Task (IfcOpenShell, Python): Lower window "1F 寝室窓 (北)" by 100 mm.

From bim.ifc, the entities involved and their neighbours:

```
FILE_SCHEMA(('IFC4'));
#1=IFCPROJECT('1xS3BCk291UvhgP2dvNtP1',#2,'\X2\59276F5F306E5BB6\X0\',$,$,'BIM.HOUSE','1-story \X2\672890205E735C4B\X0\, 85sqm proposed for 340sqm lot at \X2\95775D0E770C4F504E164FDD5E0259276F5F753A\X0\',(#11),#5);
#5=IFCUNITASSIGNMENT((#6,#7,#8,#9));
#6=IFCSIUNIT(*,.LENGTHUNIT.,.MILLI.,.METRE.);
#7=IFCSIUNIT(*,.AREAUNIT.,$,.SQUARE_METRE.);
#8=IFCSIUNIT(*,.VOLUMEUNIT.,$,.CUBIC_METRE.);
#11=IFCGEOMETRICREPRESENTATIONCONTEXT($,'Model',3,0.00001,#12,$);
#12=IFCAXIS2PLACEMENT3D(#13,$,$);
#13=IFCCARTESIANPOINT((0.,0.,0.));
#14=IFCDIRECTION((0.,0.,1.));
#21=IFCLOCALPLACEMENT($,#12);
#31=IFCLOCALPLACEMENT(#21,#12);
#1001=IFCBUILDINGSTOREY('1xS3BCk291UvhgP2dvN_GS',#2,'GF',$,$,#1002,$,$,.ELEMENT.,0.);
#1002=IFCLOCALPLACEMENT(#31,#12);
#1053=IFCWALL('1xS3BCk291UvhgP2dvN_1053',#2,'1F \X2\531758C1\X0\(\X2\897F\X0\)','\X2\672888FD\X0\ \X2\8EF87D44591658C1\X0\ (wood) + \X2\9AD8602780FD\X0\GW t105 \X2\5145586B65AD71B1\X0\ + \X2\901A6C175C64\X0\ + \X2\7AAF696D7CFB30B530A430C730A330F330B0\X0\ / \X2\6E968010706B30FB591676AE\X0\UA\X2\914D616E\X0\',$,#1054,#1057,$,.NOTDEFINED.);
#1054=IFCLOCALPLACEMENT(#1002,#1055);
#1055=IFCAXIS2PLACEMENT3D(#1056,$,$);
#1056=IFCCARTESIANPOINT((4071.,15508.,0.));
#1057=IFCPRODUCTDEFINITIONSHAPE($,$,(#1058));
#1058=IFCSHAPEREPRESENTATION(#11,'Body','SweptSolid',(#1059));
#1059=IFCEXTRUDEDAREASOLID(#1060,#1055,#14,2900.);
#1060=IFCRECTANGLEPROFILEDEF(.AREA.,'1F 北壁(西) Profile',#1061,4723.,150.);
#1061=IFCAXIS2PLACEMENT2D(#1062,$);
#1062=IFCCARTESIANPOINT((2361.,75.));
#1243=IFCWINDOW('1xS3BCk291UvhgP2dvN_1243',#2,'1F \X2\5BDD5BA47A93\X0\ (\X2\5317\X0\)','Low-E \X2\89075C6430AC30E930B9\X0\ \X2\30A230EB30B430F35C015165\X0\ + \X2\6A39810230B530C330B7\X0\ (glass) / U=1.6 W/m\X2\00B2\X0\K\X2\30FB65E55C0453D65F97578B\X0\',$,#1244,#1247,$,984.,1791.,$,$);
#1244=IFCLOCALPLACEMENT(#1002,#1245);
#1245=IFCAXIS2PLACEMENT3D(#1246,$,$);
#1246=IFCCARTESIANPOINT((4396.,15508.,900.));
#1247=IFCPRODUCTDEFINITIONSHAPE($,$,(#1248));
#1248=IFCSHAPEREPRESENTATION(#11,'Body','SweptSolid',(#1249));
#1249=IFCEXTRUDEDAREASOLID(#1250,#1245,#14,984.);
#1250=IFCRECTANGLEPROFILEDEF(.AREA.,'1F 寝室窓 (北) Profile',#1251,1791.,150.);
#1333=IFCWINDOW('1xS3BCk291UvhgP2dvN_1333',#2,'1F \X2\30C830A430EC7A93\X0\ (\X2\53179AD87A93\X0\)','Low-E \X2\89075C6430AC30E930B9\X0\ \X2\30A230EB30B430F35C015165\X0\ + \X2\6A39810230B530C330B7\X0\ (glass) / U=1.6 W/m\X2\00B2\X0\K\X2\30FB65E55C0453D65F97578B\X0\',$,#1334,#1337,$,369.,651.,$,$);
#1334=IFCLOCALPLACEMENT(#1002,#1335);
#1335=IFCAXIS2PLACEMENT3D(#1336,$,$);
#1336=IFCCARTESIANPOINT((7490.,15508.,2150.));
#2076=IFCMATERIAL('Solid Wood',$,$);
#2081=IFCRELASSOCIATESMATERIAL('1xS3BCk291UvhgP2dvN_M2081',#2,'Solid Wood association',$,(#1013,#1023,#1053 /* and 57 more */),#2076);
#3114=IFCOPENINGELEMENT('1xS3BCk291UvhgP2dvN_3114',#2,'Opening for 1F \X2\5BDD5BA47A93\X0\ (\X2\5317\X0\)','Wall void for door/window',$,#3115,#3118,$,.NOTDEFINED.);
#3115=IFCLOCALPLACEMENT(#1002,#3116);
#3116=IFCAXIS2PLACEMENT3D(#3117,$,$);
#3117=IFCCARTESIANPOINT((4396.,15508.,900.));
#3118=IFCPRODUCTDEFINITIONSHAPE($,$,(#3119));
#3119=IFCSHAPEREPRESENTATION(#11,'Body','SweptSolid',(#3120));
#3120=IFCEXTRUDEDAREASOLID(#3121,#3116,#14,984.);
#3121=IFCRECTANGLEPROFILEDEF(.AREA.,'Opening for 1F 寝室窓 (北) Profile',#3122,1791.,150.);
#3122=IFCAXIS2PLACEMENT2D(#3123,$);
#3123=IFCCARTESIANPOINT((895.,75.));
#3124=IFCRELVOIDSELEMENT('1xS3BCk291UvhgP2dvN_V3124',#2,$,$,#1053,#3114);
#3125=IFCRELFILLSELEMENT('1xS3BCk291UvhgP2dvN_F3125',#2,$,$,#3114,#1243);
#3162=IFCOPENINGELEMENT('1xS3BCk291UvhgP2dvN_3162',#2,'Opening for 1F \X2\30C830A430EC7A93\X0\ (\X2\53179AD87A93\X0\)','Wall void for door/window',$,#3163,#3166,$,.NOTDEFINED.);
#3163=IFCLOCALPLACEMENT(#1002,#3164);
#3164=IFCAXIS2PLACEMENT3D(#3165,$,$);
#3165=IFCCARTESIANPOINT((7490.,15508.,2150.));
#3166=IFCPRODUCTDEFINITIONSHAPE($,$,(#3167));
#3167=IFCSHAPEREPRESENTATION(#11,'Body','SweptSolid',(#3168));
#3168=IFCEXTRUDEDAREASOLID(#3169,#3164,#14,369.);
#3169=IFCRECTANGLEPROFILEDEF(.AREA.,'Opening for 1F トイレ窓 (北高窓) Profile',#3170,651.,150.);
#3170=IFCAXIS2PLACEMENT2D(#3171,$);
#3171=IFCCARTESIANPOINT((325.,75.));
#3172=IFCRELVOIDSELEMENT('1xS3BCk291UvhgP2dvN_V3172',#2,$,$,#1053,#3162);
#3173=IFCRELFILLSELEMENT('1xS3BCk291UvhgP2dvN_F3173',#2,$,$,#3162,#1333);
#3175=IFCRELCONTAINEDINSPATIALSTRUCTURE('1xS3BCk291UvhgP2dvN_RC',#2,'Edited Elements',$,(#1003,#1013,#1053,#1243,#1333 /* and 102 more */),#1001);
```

```python
import numpy as np
import ifcopenshell
import ifcopenshell.api.geometry
import ifcopenshell.util.placement
import ifcopenshell.util.unit

model = ifcopenshell.open("bim.ifc")
unit_scale = ifcopenshell.util.unit.calculate_unit_scale(model)

window = model.by_guid("1xS3BCk291UvhgP2dvN_1243")
opening = window.FillsVoids[0].RelatingOpeningElement
dz = -100.0

shift = np.array([0.0, 0.0, dz])
# The window is not placed relative to its opening, so move both.
for product in (opening, window):
    matrix = ifcopenshell.util.placement.get_local_placement(product.ObjectPlacement)
    matrix[:3, 3] += shift
    ifcopenshell.api.geometry.edit_object_placement(model, product=product, matrix=matrix, is_si=False)

print(f"moved by {dz * unit_scale:+.3f} m")

model.write("bim_updated.ifc")
```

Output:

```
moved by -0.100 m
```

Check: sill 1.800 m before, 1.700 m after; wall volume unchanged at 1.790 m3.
